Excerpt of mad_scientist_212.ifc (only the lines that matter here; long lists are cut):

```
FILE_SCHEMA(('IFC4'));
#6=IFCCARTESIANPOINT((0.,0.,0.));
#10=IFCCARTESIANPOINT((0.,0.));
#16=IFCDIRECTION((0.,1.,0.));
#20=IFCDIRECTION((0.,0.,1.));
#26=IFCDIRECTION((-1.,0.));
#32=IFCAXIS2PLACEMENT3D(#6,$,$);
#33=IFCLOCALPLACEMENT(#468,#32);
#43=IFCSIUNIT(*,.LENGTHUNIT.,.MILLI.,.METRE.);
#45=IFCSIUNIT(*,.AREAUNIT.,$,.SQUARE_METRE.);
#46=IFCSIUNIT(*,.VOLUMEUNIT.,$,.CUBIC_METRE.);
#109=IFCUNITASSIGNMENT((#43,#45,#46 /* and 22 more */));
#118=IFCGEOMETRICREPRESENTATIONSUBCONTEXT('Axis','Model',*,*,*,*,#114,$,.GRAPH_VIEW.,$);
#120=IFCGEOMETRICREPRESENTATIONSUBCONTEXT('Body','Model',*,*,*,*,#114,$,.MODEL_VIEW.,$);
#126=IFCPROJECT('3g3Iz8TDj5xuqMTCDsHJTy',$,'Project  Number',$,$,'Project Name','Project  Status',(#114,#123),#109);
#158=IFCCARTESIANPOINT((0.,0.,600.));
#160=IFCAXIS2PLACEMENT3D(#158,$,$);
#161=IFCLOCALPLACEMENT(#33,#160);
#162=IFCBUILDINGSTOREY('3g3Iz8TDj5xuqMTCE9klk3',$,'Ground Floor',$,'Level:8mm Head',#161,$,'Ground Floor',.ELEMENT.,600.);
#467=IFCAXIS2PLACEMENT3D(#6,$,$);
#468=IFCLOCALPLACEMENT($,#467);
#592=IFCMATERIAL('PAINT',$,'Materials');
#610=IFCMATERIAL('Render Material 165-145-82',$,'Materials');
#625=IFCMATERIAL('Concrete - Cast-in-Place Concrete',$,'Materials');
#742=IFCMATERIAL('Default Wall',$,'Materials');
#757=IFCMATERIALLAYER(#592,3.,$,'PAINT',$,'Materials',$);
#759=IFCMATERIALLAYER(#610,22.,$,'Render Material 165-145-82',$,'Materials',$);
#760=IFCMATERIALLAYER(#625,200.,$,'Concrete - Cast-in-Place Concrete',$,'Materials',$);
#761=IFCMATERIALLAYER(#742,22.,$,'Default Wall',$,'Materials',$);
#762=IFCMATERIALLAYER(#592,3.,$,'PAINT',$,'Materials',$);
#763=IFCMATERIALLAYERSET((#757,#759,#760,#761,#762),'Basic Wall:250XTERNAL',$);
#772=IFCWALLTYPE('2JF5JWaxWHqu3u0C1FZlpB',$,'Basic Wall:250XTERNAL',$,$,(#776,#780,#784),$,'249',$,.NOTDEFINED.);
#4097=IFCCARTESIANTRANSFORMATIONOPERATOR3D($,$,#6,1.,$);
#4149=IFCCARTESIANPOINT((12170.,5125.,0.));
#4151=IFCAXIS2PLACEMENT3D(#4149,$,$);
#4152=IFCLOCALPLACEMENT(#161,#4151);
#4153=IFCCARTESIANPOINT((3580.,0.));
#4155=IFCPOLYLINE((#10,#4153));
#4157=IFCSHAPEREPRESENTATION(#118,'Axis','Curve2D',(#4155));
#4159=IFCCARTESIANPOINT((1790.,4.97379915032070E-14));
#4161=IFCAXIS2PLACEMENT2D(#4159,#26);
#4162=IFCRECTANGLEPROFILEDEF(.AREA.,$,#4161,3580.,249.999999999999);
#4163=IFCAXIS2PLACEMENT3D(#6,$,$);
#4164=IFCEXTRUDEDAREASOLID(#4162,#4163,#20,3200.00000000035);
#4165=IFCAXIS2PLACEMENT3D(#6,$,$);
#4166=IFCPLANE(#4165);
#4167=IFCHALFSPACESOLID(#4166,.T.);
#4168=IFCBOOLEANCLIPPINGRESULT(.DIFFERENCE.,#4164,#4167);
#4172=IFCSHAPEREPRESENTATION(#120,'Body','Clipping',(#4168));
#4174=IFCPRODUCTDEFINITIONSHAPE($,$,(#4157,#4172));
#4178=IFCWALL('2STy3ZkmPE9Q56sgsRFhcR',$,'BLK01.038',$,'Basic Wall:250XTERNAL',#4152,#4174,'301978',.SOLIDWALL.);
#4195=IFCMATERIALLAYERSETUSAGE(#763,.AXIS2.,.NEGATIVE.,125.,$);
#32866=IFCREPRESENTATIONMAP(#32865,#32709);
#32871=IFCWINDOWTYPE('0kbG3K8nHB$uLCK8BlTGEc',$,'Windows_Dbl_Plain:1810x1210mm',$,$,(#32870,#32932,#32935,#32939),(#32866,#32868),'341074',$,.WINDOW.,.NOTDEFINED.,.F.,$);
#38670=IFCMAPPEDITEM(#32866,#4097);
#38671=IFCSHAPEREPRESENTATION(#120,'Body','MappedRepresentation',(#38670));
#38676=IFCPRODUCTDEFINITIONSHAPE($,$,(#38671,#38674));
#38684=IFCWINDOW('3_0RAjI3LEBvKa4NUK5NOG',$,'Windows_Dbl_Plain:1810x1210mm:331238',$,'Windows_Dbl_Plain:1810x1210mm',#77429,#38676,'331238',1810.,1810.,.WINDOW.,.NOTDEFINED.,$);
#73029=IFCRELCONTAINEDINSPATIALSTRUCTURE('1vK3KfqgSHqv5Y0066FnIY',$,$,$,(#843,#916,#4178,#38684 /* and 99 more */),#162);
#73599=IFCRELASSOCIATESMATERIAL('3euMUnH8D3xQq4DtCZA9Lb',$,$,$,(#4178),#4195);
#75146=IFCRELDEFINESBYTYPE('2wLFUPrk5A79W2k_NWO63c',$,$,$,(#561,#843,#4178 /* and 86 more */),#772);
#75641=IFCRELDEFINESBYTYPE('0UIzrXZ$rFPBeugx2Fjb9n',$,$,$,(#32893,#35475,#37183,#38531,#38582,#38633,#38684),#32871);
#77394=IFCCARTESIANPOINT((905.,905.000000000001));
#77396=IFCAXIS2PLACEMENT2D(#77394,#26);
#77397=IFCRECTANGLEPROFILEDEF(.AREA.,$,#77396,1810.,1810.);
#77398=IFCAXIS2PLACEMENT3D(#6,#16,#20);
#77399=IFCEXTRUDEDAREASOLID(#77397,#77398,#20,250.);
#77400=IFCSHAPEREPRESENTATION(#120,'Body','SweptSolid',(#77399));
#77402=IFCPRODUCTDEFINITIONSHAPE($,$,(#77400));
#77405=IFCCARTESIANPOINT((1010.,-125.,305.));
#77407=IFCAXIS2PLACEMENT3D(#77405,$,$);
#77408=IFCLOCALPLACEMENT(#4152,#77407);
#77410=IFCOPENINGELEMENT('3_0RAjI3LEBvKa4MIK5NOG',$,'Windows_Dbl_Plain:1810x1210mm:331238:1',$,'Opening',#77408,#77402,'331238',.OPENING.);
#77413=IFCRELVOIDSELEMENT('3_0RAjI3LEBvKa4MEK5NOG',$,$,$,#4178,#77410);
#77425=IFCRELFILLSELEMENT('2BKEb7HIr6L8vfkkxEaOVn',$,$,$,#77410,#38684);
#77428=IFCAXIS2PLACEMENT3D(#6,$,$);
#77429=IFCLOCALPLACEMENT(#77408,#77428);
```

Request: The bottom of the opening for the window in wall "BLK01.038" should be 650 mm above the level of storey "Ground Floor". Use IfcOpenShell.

```python
import numpy as np
import ifcopenshell
import ifcopenshell.api.geometry
import ifcopenshell.geom
import ifcopenshell.util.element
import ifcopenshell.util.placement
import ifcopenshell.util.shape
import ifcopenshell.util.unit

model = ifcopenshell.open("mad_scientist_212.ifc")
unit_scale = ifcopenshell.util.unit.calculate_unit_scale(model)

window = model.by_guid("3_0RAjI3LEBvKa4NUK5NOG")
opening = window.FillsVoids[0].RelatingOpeningElement
storey = ifcopenshell.util.element.get_container(window, ifc_class="IfcBuildingStorey")
level = ifcopenshell.util.placement.get_local_placement(storey.ObjectPlacement)[2, 3]

# The opening's origin need not be at the sill, so measure its lowest point.
shape = ifcopenshell.geom.create_shape(ifcopenshell.geom.settings(), opening)
bottom = ifcopenshell.util.shape.get_shape_bottom_elevation(shape, shape.geometry) / unit_scale
dz = level + 0.65 / unit_scale - bottom

shift = np.array([0.0, 0.0, dz])
# The window is placed relative to its opening, so it follows when the opening moves.
matrix = ifcopenshell.util.placement.get_local_placement(opening.ObjectPlacement)
matrix[:3, 3] += shift
ifcopenshell.api.geometry.edit_object_placement(
    model, product=opening, matrix=matrix, is_si=False, should_transform_children=True
)

print(f"moved by {dz * unit_scale:+.3f} m")

model.write("mad_scientist_212-out.ifc")
```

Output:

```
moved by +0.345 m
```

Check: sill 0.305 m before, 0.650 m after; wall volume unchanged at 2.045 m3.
